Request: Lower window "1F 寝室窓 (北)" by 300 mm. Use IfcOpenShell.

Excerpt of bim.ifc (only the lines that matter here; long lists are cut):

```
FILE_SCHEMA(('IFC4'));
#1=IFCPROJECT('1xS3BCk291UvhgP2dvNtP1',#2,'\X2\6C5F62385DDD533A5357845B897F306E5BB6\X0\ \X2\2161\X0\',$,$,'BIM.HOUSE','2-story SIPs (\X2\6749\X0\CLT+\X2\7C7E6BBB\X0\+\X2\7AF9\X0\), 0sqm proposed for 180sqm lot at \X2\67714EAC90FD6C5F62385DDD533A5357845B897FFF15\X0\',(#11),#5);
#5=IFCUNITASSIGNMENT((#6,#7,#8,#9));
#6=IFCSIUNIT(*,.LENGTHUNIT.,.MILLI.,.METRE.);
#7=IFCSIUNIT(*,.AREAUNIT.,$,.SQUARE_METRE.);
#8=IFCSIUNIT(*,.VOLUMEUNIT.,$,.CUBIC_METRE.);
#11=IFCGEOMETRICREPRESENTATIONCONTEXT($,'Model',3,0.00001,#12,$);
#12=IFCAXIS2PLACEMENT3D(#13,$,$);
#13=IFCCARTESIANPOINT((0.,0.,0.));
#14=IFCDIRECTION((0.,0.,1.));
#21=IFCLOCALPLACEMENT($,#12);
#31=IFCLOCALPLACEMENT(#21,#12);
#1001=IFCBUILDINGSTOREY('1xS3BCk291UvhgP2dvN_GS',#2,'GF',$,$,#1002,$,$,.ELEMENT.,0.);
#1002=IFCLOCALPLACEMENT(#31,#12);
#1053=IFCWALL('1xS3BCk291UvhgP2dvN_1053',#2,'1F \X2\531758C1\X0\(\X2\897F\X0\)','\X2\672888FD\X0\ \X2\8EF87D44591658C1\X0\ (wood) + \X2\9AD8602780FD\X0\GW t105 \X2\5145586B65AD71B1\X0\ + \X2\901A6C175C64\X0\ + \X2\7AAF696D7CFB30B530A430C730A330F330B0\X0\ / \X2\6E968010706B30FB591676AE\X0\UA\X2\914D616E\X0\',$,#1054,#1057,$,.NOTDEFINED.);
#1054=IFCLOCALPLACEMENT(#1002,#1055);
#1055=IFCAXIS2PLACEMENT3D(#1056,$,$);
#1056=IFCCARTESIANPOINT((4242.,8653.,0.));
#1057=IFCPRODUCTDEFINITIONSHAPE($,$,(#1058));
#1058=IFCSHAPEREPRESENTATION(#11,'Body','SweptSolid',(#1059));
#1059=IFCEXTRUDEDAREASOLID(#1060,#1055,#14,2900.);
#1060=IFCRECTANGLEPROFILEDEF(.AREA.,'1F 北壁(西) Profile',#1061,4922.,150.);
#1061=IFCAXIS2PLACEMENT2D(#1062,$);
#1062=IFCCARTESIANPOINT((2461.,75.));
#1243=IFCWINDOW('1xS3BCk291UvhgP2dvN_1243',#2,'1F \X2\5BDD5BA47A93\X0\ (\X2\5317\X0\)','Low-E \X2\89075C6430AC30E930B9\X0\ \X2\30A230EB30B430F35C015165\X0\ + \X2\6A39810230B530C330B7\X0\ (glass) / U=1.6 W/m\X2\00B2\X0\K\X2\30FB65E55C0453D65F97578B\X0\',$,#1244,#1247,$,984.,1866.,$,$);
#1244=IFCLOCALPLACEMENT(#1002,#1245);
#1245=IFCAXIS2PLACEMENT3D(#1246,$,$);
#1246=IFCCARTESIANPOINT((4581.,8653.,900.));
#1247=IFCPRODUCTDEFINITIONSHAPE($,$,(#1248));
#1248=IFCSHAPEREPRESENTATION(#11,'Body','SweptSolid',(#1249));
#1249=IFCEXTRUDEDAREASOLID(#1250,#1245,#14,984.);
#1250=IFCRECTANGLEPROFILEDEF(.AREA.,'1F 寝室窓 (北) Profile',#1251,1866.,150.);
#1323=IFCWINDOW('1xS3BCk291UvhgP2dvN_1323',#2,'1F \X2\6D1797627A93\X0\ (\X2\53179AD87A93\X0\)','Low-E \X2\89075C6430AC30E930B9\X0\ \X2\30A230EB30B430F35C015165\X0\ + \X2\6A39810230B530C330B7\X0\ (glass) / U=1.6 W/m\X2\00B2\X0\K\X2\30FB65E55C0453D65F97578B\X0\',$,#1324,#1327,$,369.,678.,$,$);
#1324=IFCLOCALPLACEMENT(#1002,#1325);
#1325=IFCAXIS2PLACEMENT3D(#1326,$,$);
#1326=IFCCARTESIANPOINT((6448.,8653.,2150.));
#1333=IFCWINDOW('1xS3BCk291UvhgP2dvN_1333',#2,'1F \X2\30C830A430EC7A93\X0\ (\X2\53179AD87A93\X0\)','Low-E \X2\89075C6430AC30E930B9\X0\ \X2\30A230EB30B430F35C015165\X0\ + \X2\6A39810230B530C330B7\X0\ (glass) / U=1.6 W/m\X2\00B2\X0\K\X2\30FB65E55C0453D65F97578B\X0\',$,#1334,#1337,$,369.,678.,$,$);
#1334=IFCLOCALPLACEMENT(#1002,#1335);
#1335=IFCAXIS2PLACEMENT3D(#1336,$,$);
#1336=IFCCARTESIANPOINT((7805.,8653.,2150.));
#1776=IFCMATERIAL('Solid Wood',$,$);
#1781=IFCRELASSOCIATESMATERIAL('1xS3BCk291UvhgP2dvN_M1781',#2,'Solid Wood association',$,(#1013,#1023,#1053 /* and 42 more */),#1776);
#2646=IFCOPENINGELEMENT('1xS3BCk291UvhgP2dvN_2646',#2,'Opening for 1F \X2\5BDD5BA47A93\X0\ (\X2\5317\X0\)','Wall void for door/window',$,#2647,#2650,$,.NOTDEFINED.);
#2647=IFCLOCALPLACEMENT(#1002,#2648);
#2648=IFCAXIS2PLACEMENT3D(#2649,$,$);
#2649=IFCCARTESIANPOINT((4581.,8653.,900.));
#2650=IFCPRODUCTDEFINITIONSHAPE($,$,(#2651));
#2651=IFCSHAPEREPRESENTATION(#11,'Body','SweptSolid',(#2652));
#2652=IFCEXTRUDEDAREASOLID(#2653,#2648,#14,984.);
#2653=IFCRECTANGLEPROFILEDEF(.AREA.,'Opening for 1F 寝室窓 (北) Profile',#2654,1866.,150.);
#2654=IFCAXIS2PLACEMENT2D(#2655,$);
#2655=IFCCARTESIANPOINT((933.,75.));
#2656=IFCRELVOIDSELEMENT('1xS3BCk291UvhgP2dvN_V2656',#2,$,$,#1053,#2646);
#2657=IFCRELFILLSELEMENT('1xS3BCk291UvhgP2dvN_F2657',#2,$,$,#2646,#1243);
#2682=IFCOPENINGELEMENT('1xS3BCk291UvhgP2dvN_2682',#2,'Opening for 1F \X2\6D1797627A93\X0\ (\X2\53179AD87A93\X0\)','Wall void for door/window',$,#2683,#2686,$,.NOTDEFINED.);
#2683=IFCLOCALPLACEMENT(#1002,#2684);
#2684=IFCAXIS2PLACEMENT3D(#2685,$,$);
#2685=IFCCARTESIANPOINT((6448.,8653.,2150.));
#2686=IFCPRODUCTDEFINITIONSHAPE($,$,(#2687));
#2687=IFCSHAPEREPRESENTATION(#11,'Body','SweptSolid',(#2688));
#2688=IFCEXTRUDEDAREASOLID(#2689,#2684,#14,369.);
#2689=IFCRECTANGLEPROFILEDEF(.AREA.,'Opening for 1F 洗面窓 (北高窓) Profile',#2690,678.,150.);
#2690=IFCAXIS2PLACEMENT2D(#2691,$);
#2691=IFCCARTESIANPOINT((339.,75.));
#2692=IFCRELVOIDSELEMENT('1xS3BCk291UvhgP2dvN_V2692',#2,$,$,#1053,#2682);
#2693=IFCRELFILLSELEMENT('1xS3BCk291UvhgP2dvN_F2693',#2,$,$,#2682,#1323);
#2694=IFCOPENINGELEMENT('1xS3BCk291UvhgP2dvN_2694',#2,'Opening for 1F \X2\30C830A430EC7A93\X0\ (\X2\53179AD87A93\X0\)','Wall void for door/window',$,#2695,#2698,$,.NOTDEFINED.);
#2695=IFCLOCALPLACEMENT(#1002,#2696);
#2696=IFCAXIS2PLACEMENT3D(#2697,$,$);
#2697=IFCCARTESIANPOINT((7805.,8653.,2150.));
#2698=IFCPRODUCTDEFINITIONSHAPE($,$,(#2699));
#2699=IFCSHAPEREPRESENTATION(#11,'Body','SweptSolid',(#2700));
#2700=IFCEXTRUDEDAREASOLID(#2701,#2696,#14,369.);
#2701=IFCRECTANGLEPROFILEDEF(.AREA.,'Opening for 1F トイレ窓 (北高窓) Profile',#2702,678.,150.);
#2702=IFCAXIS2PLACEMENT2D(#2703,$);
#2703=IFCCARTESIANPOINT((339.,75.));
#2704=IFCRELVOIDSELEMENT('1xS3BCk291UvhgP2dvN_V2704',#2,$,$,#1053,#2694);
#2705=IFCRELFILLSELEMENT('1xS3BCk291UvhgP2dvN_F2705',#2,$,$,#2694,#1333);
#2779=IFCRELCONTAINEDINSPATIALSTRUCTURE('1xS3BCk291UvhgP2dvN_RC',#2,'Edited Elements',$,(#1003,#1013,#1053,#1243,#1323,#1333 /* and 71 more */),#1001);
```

```python
import numpy as np
import ifcopenshell
import ifcopenshell.api.geometry
import ifcopenshell.util.placement
import ifcopenshell.util.unit

model = ifcopenshell.open("bim.ifc")
unit_scale = ifcopenshell.util.unit.calculate_unit_scale(model)

window = model.by_guid("1xS3BCk291UvhgP2dvN_1243")
opening = window.FillsVoids[0].RelatingOpeningElement
dz = -0.3 / unit_scale

shift = np.array([0.0, 0.0, dz])
# The window is not placed relative to its opening, so move both.
for product in (opening, window):
    matrix = ifcopenshell.util.placement.get_local_placement(product.ObjectPlacement)
    matrix[:3, 3] += shift
    ifcopenshell.api.geometry.edit_object_placement(model, product=product, matrix=matrix, is_si=False)

print(f"moved by {dz * unit_scale:+.3f} m")

model.write("bim_v2.ifc")
```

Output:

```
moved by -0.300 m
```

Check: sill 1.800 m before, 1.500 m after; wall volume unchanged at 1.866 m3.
